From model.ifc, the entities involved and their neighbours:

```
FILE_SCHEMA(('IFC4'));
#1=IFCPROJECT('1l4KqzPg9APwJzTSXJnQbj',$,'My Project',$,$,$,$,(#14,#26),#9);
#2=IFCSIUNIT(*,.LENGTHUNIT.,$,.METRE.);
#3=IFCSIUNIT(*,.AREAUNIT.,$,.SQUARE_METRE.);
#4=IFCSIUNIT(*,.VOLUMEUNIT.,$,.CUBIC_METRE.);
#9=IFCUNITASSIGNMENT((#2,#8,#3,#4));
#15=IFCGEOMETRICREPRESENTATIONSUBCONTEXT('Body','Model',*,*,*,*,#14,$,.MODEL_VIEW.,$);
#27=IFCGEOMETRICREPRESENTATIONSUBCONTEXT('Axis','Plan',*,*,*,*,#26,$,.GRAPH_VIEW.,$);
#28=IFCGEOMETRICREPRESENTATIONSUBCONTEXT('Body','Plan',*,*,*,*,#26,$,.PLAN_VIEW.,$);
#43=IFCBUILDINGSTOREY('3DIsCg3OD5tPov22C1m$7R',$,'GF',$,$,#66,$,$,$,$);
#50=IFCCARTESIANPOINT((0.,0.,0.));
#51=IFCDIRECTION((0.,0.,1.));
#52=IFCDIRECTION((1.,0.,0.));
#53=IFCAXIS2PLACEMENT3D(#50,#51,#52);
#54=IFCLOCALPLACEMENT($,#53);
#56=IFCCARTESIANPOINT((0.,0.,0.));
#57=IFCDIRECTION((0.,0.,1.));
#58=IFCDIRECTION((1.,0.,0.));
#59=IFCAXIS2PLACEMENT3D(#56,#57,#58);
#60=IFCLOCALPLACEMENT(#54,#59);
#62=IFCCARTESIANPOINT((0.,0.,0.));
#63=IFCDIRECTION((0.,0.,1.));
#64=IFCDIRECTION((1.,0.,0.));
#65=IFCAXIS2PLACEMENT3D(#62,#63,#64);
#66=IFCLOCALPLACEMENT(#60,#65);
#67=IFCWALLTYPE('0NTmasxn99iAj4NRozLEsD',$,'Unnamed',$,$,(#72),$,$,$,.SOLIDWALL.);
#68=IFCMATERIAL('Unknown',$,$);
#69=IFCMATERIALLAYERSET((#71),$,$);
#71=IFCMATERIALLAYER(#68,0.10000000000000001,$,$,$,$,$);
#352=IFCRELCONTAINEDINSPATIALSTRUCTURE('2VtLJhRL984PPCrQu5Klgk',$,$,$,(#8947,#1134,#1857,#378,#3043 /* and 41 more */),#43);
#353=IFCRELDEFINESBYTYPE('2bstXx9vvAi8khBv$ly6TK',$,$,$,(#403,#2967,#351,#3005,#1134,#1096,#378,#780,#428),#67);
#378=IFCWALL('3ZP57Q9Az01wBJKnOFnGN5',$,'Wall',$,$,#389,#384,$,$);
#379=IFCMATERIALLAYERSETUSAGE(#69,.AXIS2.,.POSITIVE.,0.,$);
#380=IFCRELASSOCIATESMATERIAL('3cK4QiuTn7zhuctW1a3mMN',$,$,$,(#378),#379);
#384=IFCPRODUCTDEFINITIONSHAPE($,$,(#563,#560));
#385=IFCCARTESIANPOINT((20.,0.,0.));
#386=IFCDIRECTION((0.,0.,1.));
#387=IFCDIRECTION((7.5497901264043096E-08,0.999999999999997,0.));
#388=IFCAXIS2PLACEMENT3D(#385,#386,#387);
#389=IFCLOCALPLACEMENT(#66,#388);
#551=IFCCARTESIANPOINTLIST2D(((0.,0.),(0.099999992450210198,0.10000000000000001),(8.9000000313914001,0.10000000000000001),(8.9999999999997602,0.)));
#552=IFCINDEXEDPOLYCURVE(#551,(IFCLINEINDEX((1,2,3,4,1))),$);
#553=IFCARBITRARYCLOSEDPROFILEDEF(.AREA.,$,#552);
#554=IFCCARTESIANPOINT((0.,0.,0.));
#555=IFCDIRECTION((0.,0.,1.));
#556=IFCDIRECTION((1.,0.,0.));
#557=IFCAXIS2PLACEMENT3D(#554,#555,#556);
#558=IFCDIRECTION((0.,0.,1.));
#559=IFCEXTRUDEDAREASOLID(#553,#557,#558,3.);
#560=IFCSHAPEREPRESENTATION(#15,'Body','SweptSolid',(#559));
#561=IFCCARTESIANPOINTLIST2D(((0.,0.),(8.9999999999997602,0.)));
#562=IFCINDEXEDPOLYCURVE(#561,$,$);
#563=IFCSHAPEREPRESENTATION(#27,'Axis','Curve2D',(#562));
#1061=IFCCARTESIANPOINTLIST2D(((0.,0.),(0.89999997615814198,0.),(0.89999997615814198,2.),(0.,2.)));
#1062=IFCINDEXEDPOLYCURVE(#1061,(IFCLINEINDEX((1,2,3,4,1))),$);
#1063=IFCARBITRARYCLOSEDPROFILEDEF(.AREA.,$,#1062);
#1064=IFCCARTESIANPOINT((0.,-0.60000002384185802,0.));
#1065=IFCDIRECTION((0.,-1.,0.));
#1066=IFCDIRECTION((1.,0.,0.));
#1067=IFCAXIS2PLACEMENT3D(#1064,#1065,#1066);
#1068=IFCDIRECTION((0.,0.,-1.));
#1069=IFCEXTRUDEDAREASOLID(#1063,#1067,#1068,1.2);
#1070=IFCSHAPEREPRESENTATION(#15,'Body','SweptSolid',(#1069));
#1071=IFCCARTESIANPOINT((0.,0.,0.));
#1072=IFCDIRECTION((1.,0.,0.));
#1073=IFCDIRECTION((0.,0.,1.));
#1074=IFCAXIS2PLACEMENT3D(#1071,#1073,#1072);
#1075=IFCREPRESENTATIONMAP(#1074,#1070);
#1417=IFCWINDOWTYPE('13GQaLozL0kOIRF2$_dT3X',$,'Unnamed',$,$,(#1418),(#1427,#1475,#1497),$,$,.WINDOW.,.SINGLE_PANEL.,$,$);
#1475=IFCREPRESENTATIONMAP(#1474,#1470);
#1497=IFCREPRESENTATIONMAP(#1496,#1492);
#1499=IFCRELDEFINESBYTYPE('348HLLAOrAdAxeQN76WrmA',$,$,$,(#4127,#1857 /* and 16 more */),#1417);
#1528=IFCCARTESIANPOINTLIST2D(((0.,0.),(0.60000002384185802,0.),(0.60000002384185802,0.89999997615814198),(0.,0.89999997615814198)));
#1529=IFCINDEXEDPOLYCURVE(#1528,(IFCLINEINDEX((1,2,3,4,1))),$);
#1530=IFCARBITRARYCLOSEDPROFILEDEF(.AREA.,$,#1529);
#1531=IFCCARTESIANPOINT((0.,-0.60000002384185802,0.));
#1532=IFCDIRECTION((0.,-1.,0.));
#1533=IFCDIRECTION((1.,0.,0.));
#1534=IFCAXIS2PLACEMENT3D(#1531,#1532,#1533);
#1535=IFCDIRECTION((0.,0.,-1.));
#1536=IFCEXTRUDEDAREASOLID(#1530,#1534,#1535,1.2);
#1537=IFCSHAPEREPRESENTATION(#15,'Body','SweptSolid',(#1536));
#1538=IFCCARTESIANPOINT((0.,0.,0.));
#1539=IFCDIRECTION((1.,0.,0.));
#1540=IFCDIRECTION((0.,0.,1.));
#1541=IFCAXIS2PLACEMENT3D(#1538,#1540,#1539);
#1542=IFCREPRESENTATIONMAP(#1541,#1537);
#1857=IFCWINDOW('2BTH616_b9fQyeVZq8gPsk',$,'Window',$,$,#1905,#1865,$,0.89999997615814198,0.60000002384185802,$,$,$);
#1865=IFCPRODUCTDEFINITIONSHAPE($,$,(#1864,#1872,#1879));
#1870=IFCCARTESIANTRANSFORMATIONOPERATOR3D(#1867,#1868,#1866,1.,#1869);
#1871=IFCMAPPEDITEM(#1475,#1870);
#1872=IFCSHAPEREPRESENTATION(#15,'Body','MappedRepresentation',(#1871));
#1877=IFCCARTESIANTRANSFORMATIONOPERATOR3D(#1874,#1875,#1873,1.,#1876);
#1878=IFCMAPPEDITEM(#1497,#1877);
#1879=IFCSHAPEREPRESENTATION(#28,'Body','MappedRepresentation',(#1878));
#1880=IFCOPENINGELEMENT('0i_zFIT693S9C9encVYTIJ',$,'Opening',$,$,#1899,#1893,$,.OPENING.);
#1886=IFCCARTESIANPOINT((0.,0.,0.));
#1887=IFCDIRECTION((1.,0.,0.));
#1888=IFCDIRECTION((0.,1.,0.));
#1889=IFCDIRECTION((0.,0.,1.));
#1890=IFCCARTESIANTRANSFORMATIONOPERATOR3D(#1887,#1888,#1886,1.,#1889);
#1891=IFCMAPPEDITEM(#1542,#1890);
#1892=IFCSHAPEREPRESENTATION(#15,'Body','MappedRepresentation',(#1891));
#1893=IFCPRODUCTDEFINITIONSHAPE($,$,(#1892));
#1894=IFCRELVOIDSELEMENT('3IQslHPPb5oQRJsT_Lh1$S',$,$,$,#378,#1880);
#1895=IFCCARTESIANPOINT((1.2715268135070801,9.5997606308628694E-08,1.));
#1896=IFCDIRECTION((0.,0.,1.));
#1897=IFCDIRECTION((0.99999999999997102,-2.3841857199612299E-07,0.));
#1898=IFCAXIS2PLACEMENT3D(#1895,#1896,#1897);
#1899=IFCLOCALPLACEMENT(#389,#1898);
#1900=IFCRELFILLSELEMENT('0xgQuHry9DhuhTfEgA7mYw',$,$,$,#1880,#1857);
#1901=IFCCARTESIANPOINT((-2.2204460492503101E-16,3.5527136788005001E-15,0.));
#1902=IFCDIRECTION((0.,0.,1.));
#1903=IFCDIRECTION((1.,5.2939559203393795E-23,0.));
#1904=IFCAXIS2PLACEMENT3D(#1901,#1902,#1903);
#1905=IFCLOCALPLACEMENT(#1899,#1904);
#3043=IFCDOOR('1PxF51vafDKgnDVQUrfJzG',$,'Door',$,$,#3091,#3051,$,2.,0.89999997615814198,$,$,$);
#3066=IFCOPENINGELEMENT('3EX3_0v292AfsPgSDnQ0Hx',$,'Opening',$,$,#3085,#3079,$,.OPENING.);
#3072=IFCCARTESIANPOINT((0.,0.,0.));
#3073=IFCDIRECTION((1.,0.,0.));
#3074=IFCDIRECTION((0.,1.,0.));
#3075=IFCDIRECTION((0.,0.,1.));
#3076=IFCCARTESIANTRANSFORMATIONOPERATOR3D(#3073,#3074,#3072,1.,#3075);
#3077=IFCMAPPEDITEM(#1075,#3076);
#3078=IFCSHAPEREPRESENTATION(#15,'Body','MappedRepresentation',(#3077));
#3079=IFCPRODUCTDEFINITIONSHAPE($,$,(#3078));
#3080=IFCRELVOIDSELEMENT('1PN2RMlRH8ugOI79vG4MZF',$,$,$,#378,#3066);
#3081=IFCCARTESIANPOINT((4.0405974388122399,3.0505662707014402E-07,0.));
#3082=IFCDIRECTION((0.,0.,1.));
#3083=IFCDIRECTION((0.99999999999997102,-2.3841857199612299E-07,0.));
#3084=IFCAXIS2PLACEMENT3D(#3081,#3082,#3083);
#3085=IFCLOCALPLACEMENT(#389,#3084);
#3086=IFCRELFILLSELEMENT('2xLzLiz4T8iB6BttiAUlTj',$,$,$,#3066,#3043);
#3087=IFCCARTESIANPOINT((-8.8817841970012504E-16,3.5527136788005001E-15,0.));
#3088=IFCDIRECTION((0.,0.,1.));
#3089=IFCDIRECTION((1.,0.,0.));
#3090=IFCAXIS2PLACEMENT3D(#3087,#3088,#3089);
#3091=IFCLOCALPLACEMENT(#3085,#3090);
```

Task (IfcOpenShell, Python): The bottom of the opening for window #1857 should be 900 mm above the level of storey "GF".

```python
import numpy as np
import ifcopenshell
import ifcopenshell.api.geometry
import ifcopenshell.geom
import ifcopenshell.util.element
import ifcopenshell.util.placement
import ifcopenshell.util.shape
import ifcopenshell.util.unit

model = ifcopenshell.open("model.ifc")
unit_scale = ifcopenshell.util.unit.calculate_unit_scale(model)

window = model.by_guid("2BTH616_b9fQyeVZq8gPsk")
opening = window.FillsVoids[0].RelatingOpeningElement
storey = ifcopenshell.util.element.get_container(window, ifc_class="IfcBuildingStorey")
level = ifcopenshell.util.placement.get_local_placement(storey.ObjectPlacement)[2, 3]

# The opening's origin need not be at the sill, so measure its lowest point.
shape = ifcopenshell.geom.create_shape(ifcopenshell.geom.settings(), opening)
bottom = ifcopenshell.util.shape.get_shape_bottom_elevation(shape, shape.geometry) / unit_scale
dz = level + 0.9 / unit_scale - bottom

shift = np.array([0.0, 0.0, dz])
# The window is placed relative to its opening, so it follows when the opening moves.
matrix = ifcopenshell.util.placement.get_local_placement(opening.ObjectPlacement)
matrix[:3, 3] += shift
ifcopenshell.api.geometry.edit_object_placement(
    model, product=opening, matrix=matrix, is_si=False, should_transform_children=True
)

print(f"moved by {dz * unit_scale:+.3f} m")

model.write("model_updated.ifc")
```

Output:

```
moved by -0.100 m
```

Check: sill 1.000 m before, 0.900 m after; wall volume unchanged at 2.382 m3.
